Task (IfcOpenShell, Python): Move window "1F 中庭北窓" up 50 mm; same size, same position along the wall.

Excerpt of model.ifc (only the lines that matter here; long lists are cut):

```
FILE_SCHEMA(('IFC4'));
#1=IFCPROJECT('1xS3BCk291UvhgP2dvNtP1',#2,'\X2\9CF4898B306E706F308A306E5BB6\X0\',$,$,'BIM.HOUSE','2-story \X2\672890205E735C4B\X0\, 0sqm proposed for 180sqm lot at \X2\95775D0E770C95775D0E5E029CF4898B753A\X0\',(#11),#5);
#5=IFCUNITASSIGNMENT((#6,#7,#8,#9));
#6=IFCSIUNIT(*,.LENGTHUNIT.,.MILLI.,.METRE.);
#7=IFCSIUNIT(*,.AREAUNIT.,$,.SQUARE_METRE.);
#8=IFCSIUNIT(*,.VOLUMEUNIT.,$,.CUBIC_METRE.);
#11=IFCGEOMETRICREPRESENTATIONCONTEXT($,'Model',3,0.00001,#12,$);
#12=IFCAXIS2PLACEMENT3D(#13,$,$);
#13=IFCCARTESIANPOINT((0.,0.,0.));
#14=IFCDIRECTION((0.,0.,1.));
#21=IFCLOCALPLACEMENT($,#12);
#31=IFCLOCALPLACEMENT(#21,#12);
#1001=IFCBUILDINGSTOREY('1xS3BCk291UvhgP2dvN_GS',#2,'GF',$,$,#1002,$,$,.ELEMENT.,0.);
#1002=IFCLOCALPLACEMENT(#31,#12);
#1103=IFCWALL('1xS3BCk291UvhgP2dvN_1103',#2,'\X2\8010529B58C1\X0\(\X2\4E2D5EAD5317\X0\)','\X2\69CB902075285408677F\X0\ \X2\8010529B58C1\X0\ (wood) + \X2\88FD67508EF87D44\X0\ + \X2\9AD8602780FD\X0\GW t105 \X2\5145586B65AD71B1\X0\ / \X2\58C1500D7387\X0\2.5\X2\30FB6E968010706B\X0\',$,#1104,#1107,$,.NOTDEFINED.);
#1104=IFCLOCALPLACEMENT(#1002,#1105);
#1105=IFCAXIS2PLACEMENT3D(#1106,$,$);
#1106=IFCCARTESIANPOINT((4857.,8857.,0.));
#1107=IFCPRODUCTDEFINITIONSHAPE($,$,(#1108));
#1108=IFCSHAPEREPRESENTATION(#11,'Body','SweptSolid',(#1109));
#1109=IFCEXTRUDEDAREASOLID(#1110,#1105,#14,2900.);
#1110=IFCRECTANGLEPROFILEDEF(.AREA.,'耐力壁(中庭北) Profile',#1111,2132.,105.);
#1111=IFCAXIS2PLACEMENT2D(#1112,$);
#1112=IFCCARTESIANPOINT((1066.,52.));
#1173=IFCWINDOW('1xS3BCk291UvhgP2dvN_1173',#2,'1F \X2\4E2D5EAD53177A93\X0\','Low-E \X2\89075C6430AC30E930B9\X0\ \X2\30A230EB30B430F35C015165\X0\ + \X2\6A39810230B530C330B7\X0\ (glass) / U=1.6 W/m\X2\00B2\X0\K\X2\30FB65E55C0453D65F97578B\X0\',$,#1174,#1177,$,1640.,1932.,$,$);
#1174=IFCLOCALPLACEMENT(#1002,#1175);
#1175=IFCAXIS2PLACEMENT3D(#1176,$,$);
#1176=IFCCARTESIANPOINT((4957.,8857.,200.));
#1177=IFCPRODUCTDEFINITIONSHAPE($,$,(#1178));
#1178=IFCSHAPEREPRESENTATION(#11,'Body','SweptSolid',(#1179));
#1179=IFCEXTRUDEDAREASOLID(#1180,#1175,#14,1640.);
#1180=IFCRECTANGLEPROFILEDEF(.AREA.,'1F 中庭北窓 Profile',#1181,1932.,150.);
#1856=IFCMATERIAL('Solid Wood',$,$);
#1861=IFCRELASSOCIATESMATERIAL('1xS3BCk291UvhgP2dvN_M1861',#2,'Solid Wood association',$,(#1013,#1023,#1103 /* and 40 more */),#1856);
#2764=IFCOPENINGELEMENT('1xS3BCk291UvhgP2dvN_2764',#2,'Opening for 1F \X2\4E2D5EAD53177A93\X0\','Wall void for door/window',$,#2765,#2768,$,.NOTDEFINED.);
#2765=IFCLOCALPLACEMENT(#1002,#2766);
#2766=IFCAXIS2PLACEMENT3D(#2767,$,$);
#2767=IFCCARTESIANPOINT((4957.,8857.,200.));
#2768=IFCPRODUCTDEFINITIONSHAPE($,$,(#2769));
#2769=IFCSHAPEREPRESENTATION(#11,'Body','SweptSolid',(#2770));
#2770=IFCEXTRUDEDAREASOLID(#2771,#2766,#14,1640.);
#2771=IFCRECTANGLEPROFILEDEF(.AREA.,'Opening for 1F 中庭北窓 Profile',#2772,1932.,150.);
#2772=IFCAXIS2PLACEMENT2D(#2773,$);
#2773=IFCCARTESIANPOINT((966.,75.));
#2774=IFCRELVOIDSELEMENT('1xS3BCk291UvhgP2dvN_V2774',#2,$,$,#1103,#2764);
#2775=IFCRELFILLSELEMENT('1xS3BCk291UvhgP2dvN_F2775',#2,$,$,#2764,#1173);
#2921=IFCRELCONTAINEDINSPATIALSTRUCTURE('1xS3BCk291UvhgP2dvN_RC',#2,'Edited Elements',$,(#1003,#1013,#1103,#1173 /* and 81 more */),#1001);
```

```python
import numpy as np
import ifcopenshell
import ifcopenshell.api.geometry
import ifcopenshell.util.placement
import ifcopenshell.util.unit

model = ifcopenshell.open("model.ifc")
unit_scale = ifcopenshell.util.unit.calculate_unit_scale(model)

window = model.by_id(1173)
opening = window.FillsVoids[0].RelatingOpeningElement
dz = 0.05 / unit_scale

shift = np.array([0.0, 0.0, dz])
# The window is not placed relative to its opening, so move both.
for product in (opening, window):
    matrix = ifcopenshell.util.placement.get_local_placement(product.ObjectPlacement)
    matrix[:3, 3] += shift
    ifcopenshell.api.geometry.edit_object_placement(model, product=product, matrix=matrix, is_si=False)

print(f"moved by {dz * unit_scale:+.3f} m")

model.write("model_v2.ifc")
```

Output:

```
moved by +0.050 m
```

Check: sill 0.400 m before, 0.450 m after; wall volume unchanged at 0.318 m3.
